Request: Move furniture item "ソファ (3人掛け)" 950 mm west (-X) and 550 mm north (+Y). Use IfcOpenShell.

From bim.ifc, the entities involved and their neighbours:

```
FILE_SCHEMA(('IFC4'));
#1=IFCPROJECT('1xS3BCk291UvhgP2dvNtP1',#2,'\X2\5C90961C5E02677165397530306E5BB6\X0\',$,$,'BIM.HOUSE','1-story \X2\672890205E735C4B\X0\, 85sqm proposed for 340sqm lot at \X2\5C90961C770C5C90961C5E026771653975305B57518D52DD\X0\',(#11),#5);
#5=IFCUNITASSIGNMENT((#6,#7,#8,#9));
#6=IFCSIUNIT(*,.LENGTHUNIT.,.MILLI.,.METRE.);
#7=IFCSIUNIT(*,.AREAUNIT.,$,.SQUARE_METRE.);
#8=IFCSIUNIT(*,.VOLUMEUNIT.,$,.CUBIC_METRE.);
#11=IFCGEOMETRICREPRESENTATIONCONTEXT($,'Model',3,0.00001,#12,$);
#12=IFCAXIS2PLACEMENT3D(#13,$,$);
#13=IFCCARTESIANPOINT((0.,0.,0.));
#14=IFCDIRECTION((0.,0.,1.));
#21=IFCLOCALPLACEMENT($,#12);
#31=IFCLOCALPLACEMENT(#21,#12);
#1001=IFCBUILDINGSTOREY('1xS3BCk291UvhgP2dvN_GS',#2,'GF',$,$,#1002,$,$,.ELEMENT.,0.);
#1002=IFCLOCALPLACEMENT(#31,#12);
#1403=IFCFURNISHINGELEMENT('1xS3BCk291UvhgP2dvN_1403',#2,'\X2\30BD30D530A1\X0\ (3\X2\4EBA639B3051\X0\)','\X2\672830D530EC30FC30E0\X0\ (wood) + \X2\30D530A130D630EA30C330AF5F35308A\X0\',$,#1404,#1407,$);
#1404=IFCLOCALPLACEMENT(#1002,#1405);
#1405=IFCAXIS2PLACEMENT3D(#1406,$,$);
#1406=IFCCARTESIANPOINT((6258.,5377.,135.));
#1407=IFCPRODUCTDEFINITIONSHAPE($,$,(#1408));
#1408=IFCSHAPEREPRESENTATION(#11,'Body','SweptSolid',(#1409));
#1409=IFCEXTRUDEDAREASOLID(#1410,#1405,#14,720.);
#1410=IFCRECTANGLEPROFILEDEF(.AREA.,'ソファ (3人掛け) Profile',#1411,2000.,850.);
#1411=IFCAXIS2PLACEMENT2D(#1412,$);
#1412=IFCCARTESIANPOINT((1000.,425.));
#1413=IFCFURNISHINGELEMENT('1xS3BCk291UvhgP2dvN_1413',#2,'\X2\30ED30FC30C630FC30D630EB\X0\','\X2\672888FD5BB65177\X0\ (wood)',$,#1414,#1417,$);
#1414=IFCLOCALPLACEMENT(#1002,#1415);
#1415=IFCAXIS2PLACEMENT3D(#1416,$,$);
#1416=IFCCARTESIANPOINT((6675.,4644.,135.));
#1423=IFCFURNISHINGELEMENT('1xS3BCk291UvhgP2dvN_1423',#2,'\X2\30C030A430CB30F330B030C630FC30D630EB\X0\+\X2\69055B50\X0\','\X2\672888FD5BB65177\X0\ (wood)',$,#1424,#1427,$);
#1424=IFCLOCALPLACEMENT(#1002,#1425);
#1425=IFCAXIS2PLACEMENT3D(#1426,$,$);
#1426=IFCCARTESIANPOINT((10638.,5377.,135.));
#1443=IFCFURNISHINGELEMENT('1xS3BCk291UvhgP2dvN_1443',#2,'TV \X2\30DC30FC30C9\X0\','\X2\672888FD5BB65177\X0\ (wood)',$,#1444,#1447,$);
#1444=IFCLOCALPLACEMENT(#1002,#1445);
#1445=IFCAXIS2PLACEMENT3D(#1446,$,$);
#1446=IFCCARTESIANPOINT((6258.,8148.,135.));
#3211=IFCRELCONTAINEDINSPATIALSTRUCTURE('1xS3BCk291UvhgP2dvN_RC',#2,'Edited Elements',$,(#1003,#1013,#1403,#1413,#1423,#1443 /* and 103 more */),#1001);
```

```python
import ifcopenshell
import ifcopenshell.api.geometry
import ifcopenshell.util.placement
import ifcopenshell.util.unit

model = ifcopenshell.open("bim.ifc")
unit_scale = ifcopenshell.util.unit.calculate_unit_scale(model)

item = model.by_guid("1xS3BCk291UvhgP2dvN_1403")
matrix = ifcopenshell.util.placement.get_local_placement(item.ObjectPlacement)
matrix[0, 3] -= 0.95 / unit_scale
matrix[1, 3] += 0.55 / unit_scale
ifcopenshell.api.geometry.edit_object_placement(model, product=item, matrix=matrix, is_si=False)

print(ifcopenshell.util.placement.get_local_placement(item.ObjectPlacement).round(3) + 0.0)

model.write("bim_rev.ifc")
```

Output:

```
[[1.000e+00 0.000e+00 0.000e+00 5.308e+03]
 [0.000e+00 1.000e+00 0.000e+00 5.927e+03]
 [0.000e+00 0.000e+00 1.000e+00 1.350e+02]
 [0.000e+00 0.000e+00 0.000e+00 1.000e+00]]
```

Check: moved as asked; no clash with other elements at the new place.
